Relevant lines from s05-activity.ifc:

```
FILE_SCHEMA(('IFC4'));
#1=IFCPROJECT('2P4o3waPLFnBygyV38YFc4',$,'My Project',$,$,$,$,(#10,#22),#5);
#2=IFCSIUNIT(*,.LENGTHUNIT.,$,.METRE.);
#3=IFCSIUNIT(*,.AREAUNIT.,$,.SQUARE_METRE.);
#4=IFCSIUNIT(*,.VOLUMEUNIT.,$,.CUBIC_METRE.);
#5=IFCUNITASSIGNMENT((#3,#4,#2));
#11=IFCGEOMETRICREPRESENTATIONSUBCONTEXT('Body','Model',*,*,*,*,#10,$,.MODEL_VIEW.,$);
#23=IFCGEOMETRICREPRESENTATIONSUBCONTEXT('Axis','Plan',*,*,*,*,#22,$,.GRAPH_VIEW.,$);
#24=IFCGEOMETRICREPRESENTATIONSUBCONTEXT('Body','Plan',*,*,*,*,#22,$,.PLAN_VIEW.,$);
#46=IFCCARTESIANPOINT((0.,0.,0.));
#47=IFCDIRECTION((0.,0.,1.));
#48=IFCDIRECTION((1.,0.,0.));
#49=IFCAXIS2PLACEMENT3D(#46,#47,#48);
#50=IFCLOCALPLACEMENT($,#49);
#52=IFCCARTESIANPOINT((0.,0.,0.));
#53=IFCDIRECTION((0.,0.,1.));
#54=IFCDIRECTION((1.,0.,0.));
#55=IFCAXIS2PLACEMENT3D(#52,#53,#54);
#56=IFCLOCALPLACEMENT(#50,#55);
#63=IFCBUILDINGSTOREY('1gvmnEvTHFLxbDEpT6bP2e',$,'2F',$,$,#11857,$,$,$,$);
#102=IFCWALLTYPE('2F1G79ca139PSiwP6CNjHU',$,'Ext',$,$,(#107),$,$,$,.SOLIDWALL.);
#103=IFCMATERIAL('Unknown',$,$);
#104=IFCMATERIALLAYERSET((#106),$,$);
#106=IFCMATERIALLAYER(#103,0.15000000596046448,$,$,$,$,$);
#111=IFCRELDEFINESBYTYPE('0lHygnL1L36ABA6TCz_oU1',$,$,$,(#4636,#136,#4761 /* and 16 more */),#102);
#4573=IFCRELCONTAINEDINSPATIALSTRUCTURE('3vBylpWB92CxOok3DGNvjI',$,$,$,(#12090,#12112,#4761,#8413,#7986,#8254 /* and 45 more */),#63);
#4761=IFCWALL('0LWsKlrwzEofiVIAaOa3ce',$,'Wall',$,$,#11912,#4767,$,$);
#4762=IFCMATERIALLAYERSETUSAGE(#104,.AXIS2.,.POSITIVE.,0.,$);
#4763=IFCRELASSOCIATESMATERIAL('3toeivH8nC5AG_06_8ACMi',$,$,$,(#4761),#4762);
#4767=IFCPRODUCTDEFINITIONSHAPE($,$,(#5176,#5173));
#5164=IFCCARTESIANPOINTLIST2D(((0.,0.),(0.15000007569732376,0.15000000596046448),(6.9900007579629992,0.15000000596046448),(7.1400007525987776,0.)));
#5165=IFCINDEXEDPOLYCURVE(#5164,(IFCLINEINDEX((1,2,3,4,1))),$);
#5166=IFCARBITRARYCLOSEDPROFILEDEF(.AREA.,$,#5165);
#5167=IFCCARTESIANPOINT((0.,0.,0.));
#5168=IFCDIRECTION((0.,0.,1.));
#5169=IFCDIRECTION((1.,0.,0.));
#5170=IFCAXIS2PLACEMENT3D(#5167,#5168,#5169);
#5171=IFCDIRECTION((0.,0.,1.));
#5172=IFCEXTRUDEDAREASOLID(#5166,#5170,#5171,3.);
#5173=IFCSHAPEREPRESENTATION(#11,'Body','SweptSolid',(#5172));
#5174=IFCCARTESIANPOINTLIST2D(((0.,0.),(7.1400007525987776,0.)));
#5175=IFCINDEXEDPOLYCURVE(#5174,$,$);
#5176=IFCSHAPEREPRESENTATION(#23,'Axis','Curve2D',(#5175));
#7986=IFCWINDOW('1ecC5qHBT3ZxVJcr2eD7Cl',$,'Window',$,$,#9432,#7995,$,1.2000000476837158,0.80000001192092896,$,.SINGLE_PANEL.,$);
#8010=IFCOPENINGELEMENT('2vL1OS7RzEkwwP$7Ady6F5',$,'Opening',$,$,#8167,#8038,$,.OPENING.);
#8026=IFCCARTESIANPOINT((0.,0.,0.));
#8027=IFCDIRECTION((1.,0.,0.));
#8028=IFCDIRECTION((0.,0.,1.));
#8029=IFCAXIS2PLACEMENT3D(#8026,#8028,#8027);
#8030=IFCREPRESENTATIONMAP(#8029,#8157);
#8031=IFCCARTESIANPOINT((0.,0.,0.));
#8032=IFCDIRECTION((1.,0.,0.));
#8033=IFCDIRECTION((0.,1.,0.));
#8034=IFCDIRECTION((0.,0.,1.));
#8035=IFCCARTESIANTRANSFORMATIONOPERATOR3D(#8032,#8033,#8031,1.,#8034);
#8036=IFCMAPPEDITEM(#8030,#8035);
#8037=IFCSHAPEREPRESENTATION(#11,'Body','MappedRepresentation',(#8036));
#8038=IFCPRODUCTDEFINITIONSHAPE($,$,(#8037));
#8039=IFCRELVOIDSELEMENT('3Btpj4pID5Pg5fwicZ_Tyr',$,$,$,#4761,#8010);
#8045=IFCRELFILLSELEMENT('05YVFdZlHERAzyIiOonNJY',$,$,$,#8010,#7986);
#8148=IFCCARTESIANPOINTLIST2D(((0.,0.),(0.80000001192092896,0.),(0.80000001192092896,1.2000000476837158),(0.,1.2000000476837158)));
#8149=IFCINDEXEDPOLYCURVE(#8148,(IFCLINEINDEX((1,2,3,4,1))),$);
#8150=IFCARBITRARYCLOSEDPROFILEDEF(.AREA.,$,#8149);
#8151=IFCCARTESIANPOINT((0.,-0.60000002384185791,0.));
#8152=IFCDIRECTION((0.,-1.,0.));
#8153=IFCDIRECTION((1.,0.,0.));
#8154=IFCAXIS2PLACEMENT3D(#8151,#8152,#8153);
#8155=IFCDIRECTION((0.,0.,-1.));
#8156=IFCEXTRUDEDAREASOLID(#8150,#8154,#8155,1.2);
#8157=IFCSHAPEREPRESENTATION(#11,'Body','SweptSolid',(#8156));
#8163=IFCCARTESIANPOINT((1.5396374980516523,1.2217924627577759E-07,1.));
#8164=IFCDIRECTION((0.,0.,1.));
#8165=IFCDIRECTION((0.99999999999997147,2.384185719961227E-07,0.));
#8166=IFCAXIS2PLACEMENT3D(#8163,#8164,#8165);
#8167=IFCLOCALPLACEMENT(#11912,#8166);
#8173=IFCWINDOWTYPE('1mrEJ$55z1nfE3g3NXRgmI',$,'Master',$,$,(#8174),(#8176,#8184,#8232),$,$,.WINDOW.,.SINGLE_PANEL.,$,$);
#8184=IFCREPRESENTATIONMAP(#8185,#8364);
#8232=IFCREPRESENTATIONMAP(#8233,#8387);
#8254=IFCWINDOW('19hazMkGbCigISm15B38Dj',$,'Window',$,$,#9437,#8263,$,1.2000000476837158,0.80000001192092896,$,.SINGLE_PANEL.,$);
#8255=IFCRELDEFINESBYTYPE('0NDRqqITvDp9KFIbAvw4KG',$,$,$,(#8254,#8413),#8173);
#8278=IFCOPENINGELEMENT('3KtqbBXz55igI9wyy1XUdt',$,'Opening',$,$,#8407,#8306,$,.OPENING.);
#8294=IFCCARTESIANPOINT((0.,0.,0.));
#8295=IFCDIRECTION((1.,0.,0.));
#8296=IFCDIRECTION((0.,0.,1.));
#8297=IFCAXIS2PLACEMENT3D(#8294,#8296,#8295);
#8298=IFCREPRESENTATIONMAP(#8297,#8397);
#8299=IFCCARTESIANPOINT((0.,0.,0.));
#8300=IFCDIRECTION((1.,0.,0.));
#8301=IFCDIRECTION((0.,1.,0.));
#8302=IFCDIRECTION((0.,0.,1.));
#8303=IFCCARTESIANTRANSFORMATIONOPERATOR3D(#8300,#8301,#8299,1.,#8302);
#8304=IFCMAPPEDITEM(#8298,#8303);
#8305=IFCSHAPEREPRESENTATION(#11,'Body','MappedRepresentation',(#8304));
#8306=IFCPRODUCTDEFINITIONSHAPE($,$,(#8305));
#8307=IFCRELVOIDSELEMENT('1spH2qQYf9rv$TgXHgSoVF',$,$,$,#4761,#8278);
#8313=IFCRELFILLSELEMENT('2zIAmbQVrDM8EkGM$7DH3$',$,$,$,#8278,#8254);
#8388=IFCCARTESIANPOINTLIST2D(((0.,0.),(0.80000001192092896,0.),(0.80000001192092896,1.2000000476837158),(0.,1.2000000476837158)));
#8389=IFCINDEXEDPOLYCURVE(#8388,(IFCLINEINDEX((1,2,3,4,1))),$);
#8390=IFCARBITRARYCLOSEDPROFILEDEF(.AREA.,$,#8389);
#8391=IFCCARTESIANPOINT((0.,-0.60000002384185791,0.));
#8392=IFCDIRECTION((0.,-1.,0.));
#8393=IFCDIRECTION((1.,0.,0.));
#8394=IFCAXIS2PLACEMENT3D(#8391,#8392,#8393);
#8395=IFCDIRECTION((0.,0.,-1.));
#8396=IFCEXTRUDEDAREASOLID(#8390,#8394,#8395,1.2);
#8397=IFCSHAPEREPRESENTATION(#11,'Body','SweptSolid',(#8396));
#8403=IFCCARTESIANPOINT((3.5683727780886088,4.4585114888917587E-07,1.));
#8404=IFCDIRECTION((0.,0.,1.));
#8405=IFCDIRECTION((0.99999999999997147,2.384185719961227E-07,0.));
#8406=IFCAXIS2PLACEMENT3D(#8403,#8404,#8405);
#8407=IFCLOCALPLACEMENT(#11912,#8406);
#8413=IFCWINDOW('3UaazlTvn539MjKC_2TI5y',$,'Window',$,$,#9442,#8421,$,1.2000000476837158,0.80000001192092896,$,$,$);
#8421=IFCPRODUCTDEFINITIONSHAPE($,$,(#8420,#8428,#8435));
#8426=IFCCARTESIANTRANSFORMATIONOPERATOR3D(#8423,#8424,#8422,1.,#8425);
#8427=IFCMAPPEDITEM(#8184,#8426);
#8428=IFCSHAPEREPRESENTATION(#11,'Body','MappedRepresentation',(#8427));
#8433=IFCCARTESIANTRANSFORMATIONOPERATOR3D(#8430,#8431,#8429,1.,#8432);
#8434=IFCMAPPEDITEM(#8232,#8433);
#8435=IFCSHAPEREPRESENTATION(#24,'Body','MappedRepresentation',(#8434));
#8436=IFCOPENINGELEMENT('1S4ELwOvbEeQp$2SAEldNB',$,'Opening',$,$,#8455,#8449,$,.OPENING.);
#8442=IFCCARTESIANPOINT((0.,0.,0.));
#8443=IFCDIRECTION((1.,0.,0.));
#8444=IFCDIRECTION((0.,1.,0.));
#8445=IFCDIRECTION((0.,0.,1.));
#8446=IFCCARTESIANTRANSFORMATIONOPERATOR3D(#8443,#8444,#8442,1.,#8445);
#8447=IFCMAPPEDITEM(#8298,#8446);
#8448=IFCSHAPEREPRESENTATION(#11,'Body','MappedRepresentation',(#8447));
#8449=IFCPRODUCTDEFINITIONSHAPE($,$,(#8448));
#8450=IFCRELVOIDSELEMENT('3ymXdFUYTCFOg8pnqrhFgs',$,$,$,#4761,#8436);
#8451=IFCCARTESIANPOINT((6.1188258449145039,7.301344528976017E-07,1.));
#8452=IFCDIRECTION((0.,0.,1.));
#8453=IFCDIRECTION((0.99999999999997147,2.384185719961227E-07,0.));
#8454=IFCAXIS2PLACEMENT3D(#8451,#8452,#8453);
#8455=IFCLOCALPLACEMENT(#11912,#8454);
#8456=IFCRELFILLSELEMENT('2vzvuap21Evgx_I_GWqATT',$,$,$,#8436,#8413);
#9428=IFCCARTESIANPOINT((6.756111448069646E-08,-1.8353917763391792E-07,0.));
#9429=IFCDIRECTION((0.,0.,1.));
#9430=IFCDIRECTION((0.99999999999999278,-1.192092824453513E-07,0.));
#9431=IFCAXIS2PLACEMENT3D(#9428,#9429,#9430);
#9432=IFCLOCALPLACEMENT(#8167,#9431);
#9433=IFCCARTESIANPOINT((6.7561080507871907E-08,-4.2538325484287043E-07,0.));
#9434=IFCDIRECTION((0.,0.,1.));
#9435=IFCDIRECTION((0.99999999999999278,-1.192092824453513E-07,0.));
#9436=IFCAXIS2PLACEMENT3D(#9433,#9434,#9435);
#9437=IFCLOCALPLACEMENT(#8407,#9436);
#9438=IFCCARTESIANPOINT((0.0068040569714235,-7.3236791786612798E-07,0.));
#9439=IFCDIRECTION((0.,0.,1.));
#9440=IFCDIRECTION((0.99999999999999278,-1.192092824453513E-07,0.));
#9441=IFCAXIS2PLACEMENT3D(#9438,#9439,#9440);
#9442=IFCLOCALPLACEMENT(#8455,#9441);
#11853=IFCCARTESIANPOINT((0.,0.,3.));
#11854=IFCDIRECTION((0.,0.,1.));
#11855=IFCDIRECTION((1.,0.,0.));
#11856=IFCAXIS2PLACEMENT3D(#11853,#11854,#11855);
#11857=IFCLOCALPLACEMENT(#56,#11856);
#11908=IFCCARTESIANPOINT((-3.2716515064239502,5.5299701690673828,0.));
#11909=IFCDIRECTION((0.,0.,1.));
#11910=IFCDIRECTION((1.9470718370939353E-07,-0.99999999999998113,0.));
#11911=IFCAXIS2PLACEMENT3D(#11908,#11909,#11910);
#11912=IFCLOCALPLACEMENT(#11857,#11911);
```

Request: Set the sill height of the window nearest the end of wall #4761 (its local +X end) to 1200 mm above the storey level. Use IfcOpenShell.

```python
import numpy as np
import ifcopenshell
import ifcopenshell.api.geometry
import ifcopenshell.geom
import ifcopenshell.util.element
import ifcopenshell.util.placement
import ifcopenshell.util.shape
import ifcopenshell.util.unit

model = ifcopenshell.open("s05-activity.ifc")
unit_scale = ifcopenshell.util.unit.calculate_unit_scale(model)

window = model.by_guid("3UaazlTvn539MjKC_2TI5y")
opening = window.FillsVoids[0].RelatingOpeningElement
storey = ifcopenshell.util.element.get_container(window, ifc_class="IfcBuildingStorey")
level = ifcopenshell.util.placement.get_local_placement(storey.ObjectPlacement)[2, 3]

# The opening's origin need not be at the sill, so measure its lowest point.
shape = ifcopenshell.geom.create_shape(ifcopenshell.geom.settings(), opening)
bottom = ifcopenshell.util.shape.get_shape_bottom_elevation(shape, shape.geometry) / unit_scale
dz = level + 1.2 - bottom

shift = np.array([0.0, 0.0, dz])
# The window is placed relative to its opening, so it follows when the opening moves.
matrix = ifcopenshell.util.placement.get_local_placement(opening.ObjectPlacement)
matrix[:3, 3] += shift
ifcopenshell.api.geometry.edit_object_placement(
    model, product=opening, matrix=matrix, is_si=False, should_transform_children=True
)

print(f"moved by {dz * unit_scale:+.3f} m")

model.write("s05-activity_edited.ifc")
```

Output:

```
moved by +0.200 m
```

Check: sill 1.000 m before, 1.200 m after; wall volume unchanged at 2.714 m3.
